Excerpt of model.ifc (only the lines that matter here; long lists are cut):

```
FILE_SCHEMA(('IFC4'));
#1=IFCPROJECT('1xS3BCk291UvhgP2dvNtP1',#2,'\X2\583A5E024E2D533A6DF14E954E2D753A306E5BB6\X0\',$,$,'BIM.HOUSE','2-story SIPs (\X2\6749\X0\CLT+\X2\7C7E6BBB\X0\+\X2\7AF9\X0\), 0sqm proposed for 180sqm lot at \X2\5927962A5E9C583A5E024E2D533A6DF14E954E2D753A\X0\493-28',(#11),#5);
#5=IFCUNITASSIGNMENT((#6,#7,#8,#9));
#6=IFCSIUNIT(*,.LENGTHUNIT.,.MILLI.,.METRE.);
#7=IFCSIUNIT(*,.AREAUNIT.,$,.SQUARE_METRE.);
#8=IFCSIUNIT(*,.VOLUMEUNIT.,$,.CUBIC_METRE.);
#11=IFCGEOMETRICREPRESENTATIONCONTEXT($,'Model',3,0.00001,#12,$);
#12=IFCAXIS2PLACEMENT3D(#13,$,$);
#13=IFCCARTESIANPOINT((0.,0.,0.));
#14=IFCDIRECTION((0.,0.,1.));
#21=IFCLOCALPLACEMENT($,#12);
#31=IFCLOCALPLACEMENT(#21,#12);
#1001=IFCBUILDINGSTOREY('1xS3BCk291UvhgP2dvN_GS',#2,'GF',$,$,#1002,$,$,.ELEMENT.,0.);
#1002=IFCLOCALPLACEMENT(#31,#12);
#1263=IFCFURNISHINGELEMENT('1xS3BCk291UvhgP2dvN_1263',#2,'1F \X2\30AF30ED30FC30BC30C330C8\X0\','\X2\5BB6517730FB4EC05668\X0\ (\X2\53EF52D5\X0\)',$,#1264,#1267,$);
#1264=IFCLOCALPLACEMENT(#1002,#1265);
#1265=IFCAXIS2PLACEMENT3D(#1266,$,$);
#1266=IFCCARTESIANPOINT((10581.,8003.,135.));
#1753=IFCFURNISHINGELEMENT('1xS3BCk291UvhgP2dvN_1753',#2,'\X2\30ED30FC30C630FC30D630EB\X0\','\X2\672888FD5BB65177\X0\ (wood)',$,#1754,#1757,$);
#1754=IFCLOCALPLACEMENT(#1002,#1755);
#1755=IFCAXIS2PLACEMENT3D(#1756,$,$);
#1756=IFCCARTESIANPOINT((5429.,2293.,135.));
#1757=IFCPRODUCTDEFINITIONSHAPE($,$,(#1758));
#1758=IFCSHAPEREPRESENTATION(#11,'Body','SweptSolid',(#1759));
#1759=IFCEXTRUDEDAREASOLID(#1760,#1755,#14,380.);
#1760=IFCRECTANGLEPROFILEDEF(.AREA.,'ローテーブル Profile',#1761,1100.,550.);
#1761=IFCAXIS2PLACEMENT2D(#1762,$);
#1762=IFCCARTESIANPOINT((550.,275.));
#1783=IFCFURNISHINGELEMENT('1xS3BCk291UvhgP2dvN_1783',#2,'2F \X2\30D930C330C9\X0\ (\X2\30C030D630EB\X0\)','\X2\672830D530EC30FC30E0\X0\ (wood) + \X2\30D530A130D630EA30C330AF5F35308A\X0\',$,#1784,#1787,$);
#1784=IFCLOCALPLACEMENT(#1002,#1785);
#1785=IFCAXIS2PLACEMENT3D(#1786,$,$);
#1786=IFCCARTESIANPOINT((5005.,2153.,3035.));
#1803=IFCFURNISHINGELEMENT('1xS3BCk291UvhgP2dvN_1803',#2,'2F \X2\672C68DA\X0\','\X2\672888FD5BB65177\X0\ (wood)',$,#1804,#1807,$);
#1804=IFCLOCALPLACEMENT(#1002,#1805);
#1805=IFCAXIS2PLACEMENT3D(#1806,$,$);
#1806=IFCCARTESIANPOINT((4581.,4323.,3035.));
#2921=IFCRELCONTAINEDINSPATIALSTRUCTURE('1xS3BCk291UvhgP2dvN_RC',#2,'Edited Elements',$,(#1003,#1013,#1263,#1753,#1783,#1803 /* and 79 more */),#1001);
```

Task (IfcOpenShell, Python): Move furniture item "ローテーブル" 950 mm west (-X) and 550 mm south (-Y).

```python
import ifcopenshell
import ifcopenshell.api.geometry
import ifcopenshell.util.placement
import ifcopenshell.util.unit

model = ifcopenshell.open("model.ifc")
unit_scale = ifcopenshell.util.unit.calculate_unit_scale(model)

item = model.by_guid("1xS3BCk291UvhgP2dvN_1753")
matrix = ifcopenshell.util.placement.get_local_placement(item.ObjectPlacement)
matrix[0, 3] -= 0.95 / unit_scale
matrix[1, 3] -= 0.55 / unit_scale
ifcopenshell.api.geometry.edit_object_placement(model, product=item, matrix=matrix, is_si=False)

print(ifcopenshell.util.placement.get_local_placement(item.ObjectPlacement).round(3) + 0.0)

model.write("model_edited.ifc")
```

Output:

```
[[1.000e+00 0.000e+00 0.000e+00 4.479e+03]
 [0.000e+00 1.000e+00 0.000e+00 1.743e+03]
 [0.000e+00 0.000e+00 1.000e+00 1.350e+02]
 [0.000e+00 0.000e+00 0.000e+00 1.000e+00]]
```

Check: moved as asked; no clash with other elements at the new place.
